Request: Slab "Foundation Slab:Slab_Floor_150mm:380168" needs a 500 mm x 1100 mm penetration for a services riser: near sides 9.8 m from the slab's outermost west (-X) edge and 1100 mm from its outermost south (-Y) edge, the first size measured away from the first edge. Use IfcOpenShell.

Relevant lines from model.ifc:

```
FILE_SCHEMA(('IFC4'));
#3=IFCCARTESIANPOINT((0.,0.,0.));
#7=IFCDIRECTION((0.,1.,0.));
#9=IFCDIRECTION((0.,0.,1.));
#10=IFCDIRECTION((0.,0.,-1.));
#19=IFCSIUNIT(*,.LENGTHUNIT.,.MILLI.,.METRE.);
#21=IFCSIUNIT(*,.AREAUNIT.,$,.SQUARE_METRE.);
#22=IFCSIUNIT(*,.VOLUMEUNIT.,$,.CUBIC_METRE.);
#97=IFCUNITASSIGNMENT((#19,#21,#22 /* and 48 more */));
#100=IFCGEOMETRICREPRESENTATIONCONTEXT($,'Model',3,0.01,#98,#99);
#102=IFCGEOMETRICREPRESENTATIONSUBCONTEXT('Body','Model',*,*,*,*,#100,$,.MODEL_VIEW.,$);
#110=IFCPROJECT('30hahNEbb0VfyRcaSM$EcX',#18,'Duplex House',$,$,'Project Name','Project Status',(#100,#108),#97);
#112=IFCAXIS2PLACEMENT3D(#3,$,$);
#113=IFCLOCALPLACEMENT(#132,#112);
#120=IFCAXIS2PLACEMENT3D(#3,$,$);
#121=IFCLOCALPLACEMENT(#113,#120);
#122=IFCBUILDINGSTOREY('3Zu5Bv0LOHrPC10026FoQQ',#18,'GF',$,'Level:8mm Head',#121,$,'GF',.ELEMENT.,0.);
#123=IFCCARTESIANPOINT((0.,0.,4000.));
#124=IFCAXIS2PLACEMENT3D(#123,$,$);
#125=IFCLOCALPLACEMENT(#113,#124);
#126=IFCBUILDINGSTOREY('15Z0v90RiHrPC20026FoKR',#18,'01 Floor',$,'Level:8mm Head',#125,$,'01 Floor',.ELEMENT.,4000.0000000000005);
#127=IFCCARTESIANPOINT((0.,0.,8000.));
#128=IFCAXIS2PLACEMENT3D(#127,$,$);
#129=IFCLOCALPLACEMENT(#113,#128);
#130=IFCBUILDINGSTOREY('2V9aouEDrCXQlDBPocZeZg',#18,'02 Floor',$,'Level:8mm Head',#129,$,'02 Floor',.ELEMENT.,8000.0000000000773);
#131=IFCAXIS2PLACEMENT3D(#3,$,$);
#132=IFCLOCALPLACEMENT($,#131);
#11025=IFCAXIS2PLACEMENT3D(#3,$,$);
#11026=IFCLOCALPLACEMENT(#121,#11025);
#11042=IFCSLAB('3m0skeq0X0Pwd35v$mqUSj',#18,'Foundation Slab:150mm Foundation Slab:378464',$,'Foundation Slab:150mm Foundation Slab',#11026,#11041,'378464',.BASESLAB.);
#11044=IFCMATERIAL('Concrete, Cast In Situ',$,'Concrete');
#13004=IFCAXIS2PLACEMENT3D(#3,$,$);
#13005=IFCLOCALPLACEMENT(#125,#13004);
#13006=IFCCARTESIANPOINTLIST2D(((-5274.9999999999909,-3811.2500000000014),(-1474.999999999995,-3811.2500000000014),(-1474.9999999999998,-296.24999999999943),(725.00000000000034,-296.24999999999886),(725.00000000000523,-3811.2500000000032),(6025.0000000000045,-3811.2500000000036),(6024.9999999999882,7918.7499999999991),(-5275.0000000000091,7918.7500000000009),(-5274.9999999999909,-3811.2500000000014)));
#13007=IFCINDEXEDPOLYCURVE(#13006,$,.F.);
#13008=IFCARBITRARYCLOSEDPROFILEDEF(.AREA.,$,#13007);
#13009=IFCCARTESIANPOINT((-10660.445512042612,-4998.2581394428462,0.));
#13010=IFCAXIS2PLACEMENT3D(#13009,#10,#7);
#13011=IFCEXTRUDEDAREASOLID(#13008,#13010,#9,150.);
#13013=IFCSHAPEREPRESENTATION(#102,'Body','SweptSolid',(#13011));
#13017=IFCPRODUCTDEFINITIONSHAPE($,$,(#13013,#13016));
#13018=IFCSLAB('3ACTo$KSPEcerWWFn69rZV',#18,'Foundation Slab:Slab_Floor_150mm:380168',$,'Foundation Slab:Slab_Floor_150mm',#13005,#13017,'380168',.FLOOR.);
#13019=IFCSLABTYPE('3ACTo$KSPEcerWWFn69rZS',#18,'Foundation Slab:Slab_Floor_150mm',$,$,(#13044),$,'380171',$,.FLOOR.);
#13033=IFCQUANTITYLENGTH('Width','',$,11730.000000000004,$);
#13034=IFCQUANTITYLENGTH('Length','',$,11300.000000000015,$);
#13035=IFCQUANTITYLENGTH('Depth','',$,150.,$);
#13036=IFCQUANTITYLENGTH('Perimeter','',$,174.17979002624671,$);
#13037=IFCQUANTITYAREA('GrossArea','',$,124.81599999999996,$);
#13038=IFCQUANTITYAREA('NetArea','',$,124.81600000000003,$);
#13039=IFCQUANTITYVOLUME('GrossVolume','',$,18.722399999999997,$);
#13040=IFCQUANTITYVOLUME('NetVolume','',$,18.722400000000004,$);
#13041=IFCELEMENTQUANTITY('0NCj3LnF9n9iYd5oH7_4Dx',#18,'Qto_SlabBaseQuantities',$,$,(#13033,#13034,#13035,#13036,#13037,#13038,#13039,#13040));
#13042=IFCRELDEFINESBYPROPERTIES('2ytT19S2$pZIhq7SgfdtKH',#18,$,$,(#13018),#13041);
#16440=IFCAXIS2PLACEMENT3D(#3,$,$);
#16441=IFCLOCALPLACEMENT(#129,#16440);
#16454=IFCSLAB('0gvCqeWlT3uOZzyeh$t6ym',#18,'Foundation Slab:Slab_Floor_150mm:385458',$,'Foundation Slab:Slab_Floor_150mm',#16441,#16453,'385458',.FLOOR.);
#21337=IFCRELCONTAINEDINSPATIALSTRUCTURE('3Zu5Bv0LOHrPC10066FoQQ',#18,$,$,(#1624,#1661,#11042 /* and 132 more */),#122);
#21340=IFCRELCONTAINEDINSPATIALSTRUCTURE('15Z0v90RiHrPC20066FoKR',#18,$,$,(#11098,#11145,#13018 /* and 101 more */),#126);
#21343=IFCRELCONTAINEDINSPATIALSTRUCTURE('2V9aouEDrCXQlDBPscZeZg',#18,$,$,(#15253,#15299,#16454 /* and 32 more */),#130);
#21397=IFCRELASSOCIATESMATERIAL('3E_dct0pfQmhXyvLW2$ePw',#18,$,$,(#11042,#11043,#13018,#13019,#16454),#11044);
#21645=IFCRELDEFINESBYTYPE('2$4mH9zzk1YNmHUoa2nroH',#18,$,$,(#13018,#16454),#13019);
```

```python
import numpy as np
import ifcopenshell
import ifcopenshell.api.feature
import ifcopenshell.api.geometry
import ifcopenshell.api.pset
import ifcopenshell.api.root
import ifcopenshell.geom
import ifcopenshell.util.element
import ifcopenshell.util.placement
import ifcopenshell.util.representation
import ifcopenshell.util.shape
import ifcopenshell.util.unit

model = ifcopenshell.open("model.ifc")
unit_scale = ifcopenshell.util.unit.calculate_unit_scale(model)
area_scale = ifcopenshell.util.unit.calculate_unit_scale(model, "AREAUNIT")
volume_scale = ifcopenshell.util.unit.calculate_unit_scale(model, "VOLUMEUNIT")
settings = ifcopenshell.geom.settings()


def volume(element):
    """Net volume in cubic metres, openings subtracted."""
    shape = ifcopenshell.geom.create_shape(settings, element)
    return ifcopenshell.util.shape.get_volume(shape.geometry)


slab = model.by_guid("3ACTo$KSPEcerWWFn69rZV")
before = volume(slab)

# Extent in the slab's own axes, in metres. The edges named are its -X and -Y sides.
slab_shape = ifcopenshell.geom.create_shape(settings, slab)
vertices = ifcopenshell.util.shape.get_vertices(slab_shape.geometry)
x_min, y_min, bottom = vertices.min(axis=0)
top = vertices[:, 2].max()

opening = ifcopenshell.api.root.create_entity(model, ifc_class="IfcOpeningElement", name="Services riser opening", predefined_type="OPENING")
context = ifcopenshell.util.representation.get_context(model, "Model", "Body", "MODEL_VIEW")
width, depth = 0.5, 1.1
outline = [(0.0, 0.0), (width, 0.0), (width, depth), (0.0, depth), (0.0, 0.0)]
# Overshoot both faces by 50 mm so the cut is clean.
shape = ifcopenshell.api.geometry.add_slab_representation(
    model, context=context, depth=top - bottom + 0.1, polyline=outline
)
ifcopenshell.api.geometry.assign_representation(model, product=opening, representation=shape)

matrix = ifcopenshell.util.placement.get_local_placement(slab.ObjectPlacement)
matrix[:, 3] = matrix @ np.append(np.array([x_min + 9.8, y_min + 1.1, bottom - 0.05]) / unit_scale, 1.0)
ifcopenshell.api.geometry.edit_object_placement(model, product=opening, matrix=matrix, is_si=False)
ifcopenshell.api.feature.add_feature(model, feature=opening, element=slab)

after = volume(slab)

# Update the slab's stored quantities.
qto = model.by_id(ifcopenshell.util.element.get_pset(slab, "Qto_SlabBaseQuantities", should_inherit=False)["id"])
ifcopenshell.api.pset.edit_qto(model, qto=qto, properties={
    "NetArea": after / (top - bottom) / area_scale,
    "NetVolume": after / volume_scale,
})

print(f"slab volume {before:.3f} -> {after:.3f} m3")

model.write("model_rev.ifc")
```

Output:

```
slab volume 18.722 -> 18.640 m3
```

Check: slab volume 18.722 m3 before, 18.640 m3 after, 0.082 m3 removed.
